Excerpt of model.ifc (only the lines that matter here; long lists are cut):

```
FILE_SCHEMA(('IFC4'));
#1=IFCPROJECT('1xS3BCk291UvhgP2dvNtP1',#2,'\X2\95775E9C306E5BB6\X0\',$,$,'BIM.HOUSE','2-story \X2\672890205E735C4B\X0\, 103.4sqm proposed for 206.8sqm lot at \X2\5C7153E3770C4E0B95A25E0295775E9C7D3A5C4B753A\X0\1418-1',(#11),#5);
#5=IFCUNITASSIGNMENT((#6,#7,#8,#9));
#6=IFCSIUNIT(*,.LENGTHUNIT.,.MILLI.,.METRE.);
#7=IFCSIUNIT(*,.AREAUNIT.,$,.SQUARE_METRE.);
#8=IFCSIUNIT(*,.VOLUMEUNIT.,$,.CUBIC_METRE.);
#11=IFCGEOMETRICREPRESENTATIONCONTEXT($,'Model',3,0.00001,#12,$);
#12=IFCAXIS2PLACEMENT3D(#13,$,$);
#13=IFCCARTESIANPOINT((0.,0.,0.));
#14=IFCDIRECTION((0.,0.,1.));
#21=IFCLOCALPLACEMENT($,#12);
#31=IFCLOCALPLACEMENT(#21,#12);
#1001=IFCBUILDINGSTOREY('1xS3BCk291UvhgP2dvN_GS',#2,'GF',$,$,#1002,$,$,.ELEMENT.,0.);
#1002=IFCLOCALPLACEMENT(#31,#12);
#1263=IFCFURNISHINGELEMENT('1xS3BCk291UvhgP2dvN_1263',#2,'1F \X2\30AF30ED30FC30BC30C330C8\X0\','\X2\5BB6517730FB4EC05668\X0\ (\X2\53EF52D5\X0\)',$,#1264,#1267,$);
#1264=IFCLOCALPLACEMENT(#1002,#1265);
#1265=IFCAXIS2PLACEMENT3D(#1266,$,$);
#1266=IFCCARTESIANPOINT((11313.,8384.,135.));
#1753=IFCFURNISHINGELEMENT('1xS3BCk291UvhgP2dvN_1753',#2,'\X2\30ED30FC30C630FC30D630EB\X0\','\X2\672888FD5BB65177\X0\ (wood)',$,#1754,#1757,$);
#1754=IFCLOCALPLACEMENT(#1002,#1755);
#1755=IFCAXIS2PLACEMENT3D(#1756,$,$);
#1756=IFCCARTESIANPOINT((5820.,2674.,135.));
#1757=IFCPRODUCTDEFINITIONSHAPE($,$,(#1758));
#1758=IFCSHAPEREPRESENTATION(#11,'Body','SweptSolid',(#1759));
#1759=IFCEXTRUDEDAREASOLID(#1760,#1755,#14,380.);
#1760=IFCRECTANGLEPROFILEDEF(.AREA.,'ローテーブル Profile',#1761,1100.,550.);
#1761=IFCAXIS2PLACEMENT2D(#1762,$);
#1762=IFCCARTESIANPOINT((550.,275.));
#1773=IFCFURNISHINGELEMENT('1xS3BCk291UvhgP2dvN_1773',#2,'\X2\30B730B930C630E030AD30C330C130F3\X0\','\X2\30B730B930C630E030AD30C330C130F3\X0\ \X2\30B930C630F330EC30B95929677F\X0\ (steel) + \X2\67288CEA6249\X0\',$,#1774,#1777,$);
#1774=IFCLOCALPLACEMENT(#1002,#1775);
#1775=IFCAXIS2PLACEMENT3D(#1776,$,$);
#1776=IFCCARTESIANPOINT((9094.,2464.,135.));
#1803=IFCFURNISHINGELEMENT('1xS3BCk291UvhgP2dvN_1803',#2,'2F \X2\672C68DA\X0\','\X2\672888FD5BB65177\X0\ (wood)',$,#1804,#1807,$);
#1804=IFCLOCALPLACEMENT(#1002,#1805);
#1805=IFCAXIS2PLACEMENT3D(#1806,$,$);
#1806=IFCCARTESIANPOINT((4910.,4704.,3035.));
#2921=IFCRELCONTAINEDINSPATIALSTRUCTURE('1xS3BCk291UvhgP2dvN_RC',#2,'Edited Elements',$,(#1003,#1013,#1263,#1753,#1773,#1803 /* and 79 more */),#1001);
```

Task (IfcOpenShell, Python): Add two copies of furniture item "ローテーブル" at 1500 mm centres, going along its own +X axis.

```python
import ifcopenshell
import ifcopenshell.api.geometry
import ifcopenshell.api.root
import ifcopenshell.util.element
import ifcopenshell.util.placement
import ifcopenshell.util.unit

model = ifcopenshell.open("model.ifc")
unit_scale = ifcopenshell.util.unit.calculate_unit_scale(model)


def reuse_history(source, copy):
    """copy_class also copies each property set's owner history, people and application; keep the originals."""
    for rel in copy.IsDefinedBy:
        if rel.is_a("IfcRelDefinesByProperties") and (history := rel.RelatingPropertyDefinition.OwnerHistory):
            rel.RelatingPropertyDefinition.OwnerHistory = source.OwnerHistory
            ifcopenshell.util.element.remove_deep2(model, history)


source = model.by_id(1753)
base = ifcopenshell.util.placement.get_local_placement(source.ObjectPlacement)
step = base[:3, 0] * 1.5 / unit_scale

for i in range(1, 3):
    copy = ifcopenshell.api.root.copy_class(model, product=source)
    copy.Representation = ifcopenshell.util.element.copy_deep(
        model, source.Representation, exclude=["IfcGeometricRepresentationContext", "IfcRepresentationMap"]
    )
    reuse_history(source, copy)
    matrix = base.copy()
    matrix[:3, 3] += i * step
    print("added at", matrix[:3, 3].round(3) + 0.0)
    ifcopenshell.api.geometry.edit_object_placement(model, product=copy, matrix=matrix, is_si=False)

model.write("model_edited.ifc")
```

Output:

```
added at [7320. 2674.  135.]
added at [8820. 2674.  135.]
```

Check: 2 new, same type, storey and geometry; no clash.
